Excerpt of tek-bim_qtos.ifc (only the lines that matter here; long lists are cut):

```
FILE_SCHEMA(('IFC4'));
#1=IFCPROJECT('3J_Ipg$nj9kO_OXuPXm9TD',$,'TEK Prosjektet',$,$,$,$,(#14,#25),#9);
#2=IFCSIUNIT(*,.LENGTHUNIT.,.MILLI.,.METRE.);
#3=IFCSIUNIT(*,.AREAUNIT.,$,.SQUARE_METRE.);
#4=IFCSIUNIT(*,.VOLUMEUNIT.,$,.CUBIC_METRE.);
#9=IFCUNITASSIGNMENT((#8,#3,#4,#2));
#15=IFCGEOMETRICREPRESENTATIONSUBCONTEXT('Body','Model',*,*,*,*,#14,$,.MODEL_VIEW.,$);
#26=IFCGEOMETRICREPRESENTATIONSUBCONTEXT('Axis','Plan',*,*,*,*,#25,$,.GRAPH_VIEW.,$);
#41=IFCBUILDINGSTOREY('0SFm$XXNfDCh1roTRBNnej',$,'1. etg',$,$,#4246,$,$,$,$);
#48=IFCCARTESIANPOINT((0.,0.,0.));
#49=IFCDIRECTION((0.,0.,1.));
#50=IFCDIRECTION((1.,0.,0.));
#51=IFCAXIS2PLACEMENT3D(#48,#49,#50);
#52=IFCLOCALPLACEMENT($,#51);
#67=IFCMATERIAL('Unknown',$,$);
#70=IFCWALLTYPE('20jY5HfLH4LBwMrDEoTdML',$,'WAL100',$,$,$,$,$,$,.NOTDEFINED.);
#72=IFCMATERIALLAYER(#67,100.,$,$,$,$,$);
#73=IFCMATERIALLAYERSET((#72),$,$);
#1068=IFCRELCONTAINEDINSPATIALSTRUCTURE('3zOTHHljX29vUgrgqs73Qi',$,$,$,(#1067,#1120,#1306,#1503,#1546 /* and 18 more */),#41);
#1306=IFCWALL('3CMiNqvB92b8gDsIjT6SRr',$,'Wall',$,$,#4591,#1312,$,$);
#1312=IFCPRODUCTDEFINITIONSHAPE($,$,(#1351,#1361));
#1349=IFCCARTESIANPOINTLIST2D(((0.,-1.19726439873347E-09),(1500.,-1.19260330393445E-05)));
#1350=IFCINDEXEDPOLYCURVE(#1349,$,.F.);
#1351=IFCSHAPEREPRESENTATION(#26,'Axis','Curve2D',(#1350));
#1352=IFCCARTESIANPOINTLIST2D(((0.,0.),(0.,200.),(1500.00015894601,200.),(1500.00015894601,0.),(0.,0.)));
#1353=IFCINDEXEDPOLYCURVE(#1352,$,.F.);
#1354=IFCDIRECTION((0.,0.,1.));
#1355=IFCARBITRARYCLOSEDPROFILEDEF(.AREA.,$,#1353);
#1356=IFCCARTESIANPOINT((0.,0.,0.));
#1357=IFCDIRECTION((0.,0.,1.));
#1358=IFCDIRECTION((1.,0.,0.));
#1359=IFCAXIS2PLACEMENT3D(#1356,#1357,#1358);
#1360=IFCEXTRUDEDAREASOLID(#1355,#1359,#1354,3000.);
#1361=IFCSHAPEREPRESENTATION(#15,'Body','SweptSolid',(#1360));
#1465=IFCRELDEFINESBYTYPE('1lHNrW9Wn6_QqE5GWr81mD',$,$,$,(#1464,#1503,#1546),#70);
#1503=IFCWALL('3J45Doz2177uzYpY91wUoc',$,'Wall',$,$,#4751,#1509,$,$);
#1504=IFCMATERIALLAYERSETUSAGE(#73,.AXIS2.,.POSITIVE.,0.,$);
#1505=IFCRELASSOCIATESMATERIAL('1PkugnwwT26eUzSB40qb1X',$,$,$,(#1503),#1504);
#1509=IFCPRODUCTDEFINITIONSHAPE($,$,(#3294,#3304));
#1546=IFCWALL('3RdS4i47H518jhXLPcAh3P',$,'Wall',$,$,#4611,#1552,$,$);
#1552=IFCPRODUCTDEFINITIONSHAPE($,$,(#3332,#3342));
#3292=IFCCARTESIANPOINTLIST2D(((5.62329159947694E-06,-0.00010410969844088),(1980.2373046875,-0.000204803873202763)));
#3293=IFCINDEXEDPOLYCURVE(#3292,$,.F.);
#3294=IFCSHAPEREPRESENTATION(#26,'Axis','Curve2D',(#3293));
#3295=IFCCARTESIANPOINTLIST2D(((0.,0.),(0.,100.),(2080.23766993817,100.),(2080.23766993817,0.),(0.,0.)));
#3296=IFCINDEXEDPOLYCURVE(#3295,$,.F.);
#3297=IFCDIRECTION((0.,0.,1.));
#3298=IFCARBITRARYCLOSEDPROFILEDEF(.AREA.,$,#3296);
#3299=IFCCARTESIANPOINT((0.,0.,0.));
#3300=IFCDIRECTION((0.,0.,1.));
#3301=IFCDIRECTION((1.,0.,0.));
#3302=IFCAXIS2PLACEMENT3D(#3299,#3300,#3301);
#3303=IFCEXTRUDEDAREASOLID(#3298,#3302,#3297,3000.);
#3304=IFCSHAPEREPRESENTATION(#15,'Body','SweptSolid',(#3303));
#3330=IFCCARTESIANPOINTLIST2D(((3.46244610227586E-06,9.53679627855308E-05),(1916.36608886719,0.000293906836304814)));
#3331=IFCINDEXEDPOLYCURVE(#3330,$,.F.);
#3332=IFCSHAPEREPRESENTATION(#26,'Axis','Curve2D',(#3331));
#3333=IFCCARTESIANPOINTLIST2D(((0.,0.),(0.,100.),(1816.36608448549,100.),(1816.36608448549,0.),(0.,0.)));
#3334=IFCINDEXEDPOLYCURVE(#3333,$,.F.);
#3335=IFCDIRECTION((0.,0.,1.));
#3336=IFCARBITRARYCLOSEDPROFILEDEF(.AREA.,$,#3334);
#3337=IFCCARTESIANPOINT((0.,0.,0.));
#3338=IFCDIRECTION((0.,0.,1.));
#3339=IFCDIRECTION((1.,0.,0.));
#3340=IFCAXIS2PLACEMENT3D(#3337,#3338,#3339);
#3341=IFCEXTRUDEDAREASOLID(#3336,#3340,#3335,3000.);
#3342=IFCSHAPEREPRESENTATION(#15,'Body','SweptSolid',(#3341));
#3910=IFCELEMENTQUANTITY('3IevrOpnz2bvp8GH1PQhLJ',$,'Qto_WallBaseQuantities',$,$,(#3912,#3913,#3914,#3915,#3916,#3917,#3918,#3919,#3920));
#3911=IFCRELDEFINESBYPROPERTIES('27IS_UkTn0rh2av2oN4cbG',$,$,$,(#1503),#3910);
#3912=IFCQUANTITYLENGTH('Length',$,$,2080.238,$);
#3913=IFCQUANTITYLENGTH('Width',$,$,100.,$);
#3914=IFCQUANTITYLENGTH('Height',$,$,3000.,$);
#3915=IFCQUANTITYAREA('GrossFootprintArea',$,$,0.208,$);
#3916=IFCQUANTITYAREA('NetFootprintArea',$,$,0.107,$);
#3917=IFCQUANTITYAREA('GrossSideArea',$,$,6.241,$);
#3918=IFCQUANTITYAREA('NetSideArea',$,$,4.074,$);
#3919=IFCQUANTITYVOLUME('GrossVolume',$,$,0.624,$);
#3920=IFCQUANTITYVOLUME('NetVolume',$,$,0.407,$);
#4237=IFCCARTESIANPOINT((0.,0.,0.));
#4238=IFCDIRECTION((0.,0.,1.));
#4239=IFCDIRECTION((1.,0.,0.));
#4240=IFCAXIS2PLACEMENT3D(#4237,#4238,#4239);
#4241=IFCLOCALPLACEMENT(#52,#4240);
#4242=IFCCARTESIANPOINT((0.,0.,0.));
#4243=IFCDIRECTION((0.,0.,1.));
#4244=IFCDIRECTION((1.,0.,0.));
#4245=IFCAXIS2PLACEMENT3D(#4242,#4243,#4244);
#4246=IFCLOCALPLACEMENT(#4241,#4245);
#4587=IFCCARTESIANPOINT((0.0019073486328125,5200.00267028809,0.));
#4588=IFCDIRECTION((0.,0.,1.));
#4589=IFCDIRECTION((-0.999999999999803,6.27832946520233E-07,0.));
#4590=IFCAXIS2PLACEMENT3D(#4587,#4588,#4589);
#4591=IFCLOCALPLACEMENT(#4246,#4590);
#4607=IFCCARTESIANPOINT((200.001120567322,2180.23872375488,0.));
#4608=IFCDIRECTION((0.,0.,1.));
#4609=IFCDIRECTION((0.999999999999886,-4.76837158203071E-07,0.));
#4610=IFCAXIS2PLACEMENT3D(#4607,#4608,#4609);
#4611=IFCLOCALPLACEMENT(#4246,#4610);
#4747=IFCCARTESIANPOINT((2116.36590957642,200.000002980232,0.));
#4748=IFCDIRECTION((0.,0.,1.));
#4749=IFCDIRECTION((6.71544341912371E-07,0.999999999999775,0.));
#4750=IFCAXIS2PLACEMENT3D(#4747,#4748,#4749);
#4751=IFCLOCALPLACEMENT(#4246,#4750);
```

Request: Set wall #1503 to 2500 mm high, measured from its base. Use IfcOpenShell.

```python
import ifcopenshell
import ifcopenshell.api.pset
import ifcopenshell.geom
import ifcopenshell.util.element
import ifcopenshell.util.representation
import ifcopenshell.util.shape
import ifcopenshell.util.unit

model = ifcopenshell.open("tek-bim_qtos.ifc")
unit_scale = ifcopenshell.util.unit.calculate_unit_scale(model)
area_scale = ifcopenshell.util.unit.calculate_unit_scale(model, "AREAUNIT")
volume_scale = ifcopenshell.util.unit.calculate_unit_scale(model, "VOLUMEUNIT")
settings = ifcopenshell.geom.settings()


def volume(element):
    """Net volume in cubic metres, openings subtracted."""
    shape = ifcopenshell.geom.create_shape(settings, element)
    return ifcopenshell.util.shape.get_volume(shape.geometry)


wall = model.by_id(1503)
before = volume(wall)

body = ifcopenshell.util.representation.get_representation(wall, "Model", "Body")
solid = body.Items[0]
old_height = solid.Depth
solid.Depth = 2.5 / unit_scale
after = volume(wall)
thickness = 0.1  # wall thickness in metres

# Update the stored height, areas and volumes.
qto = model.by_id(ifcopenshell.util.element.get_pset(wall, "Qto_WallBaseQuantities", should_inherit=False)["id"])
ifcopenshell.api.pset.edit_qto(model, qto=qto, properties={
    "Height": solid.Depth,
    "GrossSideArea": ifcopenshell.util.element.get_pset(wall, "Qto_WallBaseQuantities", "GrossSideArea") * solid.Depth / old_height,
    "NetSideArea": after / thickness / area_scale,
    "GrossVolume": ifcopenshell.util.element.get_pset(wall, "Qto_WallBaseQuantities", "GrossVolume") * solid.Depth / old_height,
    "NetVolume": after / volume_scale,
})

print(f"height {old_height:g} -> {solid.Depth:g}, volume {before:.3f} -> {after:.3f} m3")

model.write("tek-bim_qtos_edited.ifc")
```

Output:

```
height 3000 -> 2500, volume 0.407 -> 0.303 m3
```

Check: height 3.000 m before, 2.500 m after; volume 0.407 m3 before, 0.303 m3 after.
